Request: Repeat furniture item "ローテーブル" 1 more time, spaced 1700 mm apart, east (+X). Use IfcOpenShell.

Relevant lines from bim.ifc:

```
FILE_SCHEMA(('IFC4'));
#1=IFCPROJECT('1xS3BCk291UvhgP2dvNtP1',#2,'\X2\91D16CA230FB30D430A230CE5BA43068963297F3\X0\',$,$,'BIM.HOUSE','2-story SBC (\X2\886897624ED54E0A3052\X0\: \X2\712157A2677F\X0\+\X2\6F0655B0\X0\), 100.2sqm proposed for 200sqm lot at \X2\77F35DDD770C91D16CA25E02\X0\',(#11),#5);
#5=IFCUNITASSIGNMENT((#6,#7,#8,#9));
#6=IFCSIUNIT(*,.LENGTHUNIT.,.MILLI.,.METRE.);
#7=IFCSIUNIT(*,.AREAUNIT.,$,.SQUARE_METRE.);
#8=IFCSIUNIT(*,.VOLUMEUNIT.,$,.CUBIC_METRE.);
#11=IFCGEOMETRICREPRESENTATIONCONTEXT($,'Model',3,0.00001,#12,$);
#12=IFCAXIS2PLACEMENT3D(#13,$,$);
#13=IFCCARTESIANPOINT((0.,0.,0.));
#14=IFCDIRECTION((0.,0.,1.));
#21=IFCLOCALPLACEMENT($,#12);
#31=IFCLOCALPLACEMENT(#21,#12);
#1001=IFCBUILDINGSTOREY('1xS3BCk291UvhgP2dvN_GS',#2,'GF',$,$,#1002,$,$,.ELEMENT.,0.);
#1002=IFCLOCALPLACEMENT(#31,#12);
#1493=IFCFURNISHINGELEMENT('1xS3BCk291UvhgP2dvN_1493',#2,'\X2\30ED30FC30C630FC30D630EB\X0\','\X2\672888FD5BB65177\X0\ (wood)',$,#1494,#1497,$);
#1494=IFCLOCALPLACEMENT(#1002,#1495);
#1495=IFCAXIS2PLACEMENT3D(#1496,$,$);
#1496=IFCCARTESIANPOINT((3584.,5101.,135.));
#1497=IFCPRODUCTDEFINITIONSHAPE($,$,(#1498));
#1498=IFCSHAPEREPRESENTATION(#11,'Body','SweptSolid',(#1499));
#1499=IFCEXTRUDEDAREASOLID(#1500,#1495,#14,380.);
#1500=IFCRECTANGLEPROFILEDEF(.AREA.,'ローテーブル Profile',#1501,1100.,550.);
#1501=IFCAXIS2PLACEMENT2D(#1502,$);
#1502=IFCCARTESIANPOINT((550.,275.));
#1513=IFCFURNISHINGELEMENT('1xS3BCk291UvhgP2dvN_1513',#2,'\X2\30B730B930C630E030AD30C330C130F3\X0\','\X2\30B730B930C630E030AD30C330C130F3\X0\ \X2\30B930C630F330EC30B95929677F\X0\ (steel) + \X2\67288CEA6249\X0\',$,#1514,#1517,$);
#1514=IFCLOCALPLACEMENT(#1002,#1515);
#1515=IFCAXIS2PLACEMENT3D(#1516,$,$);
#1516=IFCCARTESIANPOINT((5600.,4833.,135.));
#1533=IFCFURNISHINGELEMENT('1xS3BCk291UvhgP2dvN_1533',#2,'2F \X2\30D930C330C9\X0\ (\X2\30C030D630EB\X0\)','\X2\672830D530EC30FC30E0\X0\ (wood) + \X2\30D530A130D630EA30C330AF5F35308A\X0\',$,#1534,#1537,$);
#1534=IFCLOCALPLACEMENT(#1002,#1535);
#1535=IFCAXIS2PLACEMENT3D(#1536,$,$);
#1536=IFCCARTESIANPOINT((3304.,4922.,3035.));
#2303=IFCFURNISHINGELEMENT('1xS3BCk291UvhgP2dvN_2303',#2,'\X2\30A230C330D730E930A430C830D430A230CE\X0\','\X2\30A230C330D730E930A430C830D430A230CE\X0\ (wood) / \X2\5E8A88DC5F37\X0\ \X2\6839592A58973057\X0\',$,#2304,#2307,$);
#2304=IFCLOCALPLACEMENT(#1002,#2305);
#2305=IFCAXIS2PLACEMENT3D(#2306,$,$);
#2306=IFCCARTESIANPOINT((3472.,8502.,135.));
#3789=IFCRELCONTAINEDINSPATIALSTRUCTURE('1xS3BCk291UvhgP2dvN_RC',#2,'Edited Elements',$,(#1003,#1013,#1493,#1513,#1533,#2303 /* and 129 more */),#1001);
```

```python
import numpy as np
import ifcopenshell
import ifcopenshell.api.geometry
import ifcopenshell.api.root
import ifcopenshell.util.element
import ifcopenshell.util.placement

model = ifcopenshell.open("bim.ifc")


def reuse_history(source, copy):
    """copy_class also copies each property set's owner history, people and application; keep the originals."""
    for rel in copy.IsDefinedBy:
        if rel.is_a("IfcRelDefinesByProperties") and (history := rel.RelatingPropertyDefinition.OwnerHistory):
            rel.RelatingPropertyDefinition.OwnerHistory = source.OwnerHistory
            ifcopenshell.util.element.remove_deep2(model, history)


source = model.by_guid("1xS3BCk291UvhgP2dvN_1493")
base = ifcopenshell.util.placement.get_local_placement(source.ObjectPlacement)
step = np.array([1.0, 0.0, 0.0]) * 1700.0

for i in range(1, 2):
    copy = ifcopenshell.api.root.copy_class(model, product=source)
    copy.Representation = ifcopenshell.util.element.copy_deep(
        model, source.Representation, exclude=["IfcGeometricRepresentationContext", "IfcRepresentationMap"]
    )
    reuse_history(source, copy)
    matrix = base.copy()
    matrix[:3, 3] += i * step
    print("added at", matrix[:3, 3].round(3) + 0.0)
    ifcopenshell.api.geometry.edit_object_placement(model, product=copy, matrix=matrix, is_si=False)

model.write("bim_rev.ifc")
```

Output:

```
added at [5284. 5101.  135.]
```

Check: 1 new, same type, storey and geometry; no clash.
